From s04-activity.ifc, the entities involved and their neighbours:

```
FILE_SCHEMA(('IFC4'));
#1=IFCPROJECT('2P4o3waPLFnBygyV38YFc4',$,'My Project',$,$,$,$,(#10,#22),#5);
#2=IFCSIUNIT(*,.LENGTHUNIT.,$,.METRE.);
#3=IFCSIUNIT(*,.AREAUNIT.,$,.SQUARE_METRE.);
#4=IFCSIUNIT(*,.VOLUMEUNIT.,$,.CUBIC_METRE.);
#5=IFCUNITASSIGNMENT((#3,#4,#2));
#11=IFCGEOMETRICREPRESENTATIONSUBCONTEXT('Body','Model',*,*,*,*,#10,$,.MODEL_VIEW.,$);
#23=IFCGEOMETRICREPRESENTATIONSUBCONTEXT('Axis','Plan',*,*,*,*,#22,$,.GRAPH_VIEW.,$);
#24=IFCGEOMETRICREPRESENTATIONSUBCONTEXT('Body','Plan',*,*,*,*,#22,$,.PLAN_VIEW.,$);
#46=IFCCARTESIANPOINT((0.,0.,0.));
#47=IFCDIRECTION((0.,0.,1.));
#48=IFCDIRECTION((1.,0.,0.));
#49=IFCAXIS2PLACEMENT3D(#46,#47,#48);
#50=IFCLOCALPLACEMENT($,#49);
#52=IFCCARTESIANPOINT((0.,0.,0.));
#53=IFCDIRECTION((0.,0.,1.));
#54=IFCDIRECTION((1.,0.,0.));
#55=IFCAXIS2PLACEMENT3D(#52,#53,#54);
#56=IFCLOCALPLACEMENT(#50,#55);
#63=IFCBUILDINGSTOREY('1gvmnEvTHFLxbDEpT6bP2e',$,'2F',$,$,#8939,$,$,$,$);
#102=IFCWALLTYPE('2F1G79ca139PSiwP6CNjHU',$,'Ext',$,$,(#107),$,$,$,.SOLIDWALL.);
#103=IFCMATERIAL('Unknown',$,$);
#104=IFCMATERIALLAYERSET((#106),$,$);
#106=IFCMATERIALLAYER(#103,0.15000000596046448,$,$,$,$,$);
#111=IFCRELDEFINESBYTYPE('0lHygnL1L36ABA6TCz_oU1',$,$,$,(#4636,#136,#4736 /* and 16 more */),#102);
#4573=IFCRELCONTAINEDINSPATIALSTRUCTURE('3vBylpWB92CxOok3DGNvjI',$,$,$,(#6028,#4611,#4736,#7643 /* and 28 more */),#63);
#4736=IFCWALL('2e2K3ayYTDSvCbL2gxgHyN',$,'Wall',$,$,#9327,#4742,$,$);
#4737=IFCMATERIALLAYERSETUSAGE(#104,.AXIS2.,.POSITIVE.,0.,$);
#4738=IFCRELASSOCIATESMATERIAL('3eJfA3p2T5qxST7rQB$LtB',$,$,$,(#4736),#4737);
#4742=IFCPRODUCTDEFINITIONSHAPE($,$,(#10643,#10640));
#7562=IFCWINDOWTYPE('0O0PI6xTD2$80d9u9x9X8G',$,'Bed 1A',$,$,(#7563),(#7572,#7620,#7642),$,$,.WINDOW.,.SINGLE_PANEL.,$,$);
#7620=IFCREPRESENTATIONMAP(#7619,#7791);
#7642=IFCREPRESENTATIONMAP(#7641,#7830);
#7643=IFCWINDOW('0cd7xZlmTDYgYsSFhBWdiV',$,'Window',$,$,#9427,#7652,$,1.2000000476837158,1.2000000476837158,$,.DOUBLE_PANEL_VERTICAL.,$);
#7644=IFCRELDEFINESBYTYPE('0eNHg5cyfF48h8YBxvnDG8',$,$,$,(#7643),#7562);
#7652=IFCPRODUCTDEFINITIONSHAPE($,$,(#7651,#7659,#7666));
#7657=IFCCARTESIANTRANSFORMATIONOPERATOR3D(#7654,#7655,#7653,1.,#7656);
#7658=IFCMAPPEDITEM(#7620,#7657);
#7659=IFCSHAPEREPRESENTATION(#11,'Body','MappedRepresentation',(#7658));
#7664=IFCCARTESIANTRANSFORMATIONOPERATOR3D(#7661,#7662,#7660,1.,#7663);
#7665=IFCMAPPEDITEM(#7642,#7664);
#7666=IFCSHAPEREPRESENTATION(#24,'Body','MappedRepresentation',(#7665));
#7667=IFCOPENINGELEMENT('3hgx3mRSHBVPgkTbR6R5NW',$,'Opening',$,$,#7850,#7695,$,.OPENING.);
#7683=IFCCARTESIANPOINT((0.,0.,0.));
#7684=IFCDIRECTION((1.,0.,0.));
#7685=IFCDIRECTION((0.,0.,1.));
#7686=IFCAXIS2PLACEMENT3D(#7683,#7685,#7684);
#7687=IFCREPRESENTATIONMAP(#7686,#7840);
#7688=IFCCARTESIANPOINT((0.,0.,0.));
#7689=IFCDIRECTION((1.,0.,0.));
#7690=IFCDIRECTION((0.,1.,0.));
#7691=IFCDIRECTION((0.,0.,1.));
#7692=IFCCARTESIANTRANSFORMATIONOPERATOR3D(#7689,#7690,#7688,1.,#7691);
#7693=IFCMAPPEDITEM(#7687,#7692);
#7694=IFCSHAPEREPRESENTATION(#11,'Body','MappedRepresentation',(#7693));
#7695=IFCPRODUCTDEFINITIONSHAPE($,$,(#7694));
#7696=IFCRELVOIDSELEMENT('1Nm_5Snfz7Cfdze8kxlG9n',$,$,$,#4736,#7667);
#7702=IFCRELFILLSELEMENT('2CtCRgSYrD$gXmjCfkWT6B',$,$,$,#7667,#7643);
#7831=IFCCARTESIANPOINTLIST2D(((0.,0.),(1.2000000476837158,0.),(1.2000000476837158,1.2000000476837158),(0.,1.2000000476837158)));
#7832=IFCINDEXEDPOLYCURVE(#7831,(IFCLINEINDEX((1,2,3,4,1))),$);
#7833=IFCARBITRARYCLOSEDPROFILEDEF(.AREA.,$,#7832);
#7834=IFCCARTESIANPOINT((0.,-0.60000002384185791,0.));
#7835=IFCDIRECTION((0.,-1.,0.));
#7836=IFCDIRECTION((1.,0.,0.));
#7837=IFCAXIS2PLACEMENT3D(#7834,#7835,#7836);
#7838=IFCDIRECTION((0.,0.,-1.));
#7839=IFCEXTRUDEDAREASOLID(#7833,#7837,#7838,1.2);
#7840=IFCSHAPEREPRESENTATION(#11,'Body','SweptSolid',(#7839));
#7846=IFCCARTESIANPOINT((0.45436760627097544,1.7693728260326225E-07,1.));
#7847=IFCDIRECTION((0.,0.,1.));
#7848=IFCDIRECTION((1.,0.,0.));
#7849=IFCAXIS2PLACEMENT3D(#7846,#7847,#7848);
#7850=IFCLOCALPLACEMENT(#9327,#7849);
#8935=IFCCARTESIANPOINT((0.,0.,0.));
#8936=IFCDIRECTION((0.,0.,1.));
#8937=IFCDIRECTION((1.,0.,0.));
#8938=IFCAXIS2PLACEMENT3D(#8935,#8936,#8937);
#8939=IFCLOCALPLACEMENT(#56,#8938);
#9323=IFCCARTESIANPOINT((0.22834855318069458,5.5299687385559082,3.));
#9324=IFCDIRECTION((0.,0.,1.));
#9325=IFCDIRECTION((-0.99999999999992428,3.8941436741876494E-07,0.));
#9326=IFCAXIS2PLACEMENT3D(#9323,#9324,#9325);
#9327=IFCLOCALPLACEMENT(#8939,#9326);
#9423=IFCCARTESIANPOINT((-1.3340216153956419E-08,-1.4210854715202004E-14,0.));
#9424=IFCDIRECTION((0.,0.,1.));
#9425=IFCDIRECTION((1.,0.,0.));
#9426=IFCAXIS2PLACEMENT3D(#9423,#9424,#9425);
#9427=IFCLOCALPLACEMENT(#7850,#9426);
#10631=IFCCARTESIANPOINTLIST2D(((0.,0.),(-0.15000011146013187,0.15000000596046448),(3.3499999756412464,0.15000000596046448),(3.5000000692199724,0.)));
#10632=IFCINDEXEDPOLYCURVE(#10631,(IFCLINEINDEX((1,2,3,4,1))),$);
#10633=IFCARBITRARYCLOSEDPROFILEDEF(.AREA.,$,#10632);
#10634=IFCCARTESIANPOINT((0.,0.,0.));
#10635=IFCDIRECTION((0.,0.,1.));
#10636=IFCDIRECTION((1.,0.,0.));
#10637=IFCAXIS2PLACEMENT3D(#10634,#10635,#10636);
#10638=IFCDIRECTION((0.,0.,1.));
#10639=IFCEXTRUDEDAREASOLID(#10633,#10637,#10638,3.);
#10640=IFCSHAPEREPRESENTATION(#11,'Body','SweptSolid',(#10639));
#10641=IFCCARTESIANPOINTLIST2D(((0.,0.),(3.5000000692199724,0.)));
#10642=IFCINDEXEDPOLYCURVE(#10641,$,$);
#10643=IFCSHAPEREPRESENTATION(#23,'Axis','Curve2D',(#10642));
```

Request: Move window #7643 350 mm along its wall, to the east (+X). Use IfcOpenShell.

```python
import ifcopenshell
import ifcopenshell.api.geometry
import ifcopenshell.util.placement
import ifcopenshell.util.unit

model = ifcopenshell.open("s04-activity.ifc")
unit_scale = ifcopenshell.util.unit.calculate_unit_scale(model)

window = model.by_guid("0cd7xZlmTDYgYsSFhBWdiV")
opening = window.FillsVoids[0].RelatingOpeningElement
wall = opening.VoidsElements[0].RelatingBuildingElement

wall_matrix = ifcopenshell.util.placement.get_local_placement(wall.ObjectPlacement)
shift = wall_matrix[:3, 0] * -0.35 / unit_scale
before = ifcopenshell.util.placement.get_local_placement(window.ObjectPlacement)[:3, 3].copy()

# The window is placed relative to its opening, so it follows when the opening moves.
matrix = ifcopenshell.util.placement.get_local_placement(opening.ObjectPlacement)
matrix[:3, 3] += shift
ifcopenshell.api.geometry.edit_object_placement(
    model, product=opening, matrix=matrix, is_si=False, should_transform_children=True
)

after = ifcopenshell.util.placement.get_local_placement(window.ObjectPlacement)[:3, 3]
print("window moved by", (after - before).round(3) + 0.0)

model.write("s04-activity_updated.ifc")
```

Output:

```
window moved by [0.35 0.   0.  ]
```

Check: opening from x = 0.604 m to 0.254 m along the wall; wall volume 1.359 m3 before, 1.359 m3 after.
